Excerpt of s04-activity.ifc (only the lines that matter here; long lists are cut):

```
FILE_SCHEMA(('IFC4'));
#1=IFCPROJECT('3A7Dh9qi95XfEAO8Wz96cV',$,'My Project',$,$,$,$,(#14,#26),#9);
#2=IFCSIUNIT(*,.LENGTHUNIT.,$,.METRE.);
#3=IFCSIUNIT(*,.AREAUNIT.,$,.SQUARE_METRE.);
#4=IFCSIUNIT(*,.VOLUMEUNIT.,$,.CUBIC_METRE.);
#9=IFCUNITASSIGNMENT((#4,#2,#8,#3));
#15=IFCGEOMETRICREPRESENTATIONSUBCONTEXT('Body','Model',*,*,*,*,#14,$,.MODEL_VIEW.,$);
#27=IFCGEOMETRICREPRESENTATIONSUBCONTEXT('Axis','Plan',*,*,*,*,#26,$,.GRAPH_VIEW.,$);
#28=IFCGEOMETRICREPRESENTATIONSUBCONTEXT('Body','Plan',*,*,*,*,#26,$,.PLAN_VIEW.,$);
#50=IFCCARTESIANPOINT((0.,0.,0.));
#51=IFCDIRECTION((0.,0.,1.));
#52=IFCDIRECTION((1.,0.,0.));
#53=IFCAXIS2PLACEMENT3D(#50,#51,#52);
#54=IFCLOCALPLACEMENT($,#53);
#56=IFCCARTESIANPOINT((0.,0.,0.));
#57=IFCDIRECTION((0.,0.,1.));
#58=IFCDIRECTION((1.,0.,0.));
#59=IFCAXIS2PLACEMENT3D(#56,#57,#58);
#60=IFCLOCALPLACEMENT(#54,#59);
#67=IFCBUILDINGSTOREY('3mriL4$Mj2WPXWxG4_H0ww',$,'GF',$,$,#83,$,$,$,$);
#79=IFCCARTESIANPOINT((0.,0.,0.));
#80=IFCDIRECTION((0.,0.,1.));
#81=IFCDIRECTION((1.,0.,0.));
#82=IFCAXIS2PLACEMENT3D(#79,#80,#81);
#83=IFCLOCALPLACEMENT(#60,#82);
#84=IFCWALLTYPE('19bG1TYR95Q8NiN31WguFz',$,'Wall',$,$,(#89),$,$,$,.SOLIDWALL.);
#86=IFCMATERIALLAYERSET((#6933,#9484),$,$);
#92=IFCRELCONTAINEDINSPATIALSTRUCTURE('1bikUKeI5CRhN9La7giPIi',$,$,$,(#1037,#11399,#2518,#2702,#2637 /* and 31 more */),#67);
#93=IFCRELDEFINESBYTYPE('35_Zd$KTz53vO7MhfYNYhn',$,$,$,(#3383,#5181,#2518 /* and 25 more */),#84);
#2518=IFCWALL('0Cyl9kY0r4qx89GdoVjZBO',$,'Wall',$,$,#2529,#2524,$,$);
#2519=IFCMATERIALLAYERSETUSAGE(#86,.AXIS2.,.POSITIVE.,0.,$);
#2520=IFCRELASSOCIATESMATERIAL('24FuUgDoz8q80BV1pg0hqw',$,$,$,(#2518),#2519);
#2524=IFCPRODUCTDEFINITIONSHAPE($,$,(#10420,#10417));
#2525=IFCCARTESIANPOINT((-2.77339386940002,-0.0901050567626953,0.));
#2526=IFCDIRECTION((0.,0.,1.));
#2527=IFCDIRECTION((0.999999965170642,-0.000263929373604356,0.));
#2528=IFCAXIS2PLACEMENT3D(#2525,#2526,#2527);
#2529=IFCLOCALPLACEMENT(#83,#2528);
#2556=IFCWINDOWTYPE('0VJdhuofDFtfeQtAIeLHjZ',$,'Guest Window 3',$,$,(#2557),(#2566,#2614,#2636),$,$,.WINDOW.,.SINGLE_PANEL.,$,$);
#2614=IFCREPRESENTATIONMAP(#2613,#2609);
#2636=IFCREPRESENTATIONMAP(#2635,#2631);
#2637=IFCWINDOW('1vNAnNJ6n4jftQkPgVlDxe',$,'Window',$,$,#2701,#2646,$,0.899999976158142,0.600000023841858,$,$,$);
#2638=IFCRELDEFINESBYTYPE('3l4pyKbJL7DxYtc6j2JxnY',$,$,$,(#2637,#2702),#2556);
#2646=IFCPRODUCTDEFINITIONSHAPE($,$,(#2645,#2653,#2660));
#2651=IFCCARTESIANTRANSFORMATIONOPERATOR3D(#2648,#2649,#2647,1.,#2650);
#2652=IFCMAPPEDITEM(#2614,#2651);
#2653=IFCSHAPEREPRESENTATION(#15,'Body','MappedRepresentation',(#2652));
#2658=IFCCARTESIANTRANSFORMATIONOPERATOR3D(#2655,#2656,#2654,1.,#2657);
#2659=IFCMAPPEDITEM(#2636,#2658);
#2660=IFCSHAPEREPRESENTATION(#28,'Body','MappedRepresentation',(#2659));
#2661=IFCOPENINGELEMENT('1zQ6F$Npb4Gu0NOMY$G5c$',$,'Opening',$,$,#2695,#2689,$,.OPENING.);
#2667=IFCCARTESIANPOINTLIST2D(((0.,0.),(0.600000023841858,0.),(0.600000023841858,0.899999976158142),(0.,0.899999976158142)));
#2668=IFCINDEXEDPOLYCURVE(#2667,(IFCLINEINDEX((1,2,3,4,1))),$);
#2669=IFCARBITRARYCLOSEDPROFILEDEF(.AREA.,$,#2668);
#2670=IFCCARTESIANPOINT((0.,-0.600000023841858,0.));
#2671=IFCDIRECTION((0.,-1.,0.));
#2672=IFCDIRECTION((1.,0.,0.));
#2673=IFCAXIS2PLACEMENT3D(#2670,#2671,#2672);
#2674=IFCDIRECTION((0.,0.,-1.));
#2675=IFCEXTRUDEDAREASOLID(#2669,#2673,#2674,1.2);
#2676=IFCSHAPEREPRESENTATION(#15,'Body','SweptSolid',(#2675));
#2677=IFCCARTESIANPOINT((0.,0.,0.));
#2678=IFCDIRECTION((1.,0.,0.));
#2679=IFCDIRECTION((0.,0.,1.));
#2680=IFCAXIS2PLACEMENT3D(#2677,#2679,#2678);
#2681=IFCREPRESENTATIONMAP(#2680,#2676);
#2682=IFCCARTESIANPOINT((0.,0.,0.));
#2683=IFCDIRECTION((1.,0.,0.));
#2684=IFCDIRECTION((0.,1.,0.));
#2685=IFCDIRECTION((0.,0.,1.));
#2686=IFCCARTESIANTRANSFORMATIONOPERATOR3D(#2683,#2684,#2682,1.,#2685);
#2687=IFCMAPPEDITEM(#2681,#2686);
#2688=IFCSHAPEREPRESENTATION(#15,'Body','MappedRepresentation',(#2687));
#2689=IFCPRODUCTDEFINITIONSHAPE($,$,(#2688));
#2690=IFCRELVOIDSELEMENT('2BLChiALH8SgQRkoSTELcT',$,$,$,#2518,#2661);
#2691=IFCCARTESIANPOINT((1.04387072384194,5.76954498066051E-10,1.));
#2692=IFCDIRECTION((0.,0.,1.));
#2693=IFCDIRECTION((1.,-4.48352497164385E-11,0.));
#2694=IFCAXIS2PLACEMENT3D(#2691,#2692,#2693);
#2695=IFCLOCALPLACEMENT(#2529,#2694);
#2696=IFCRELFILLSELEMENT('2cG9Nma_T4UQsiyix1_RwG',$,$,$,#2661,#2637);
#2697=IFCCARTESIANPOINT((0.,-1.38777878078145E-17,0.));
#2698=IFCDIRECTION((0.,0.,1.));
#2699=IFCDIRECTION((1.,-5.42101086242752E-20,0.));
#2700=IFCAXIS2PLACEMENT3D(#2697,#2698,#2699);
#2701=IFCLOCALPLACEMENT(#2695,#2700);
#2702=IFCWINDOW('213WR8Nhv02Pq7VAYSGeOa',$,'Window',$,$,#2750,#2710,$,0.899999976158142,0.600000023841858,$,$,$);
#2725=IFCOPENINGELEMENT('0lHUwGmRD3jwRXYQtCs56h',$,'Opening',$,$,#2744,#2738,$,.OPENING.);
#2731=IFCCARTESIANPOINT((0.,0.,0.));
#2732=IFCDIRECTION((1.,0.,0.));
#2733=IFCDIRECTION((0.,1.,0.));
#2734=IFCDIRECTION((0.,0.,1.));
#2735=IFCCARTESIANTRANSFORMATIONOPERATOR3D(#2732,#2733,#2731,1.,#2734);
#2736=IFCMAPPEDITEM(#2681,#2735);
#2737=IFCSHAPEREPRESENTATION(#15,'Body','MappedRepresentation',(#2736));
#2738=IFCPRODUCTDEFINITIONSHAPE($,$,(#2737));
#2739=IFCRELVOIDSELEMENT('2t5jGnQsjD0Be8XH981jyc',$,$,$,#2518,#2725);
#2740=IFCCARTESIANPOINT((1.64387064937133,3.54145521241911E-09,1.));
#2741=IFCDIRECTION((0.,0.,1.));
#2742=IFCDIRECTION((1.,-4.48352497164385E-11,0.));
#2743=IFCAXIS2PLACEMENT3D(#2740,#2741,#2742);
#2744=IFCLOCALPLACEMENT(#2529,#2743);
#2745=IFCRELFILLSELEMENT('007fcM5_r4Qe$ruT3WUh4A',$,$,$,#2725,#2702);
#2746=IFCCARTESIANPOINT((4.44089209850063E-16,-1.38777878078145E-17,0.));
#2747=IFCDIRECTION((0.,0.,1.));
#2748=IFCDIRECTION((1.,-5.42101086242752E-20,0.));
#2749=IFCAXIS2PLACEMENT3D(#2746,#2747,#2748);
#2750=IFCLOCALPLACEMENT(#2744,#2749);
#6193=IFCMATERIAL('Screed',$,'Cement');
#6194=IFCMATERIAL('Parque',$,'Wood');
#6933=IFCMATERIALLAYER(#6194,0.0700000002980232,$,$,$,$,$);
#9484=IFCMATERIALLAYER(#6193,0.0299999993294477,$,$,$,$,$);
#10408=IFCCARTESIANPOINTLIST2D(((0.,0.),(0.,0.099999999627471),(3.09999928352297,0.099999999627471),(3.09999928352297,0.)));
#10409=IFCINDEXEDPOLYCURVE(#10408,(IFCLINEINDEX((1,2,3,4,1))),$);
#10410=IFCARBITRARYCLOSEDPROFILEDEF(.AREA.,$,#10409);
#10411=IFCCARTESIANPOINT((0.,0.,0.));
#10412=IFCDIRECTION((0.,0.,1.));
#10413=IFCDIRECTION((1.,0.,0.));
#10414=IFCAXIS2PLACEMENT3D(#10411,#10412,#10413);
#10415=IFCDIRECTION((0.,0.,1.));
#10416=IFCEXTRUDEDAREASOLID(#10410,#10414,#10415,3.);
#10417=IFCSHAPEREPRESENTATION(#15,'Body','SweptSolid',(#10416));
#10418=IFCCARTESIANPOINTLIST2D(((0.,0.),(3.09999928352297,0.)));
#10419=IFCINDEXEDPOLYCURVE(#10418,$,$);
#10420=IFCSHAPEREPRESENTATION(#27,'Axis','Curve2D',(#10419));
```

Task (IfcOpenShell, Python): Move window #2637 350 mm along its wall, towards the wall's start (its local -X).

```python
import ifcopenshell
import ifcopenshell.api.geometry
import ifcopenshell.util.placement
import ifcopenshell.util.unit

model = ifcopenshell.open("s04-activity.ifc")
unit_scale = ifcopenshell.util.unit.calculate_unit_scale(model)

window = model.by_id(2637)
opening = window.FillsVoids[0].RelatingOpeningElement
wall = opening.VoidsElements[0].RelatingBuildingElement

wall_matrix = ifcopenshell.util.placement.get_local_placement(wall.ObjectPlacement)
shift = wall_matrix[:3, 0] * -0.35 / unit_scale
before = ifcopenshell.util.placement.get_local_placement(window.ObjectPlacement)[:3, 3].copy()

# The window is placed relative to its opening, so it follows when the opening moves.
matrix = ifcopenshell.util.placement.get_local_placement(opening.ObjectPlacement)
matrix[:3, 3] += shift
ifcopenshell.api.geometry.edit_object_placement(
    model, product=opening, matrix=matrix, is_si=False, should_transform_children=True
)

after = ifcopenshell.util.placement.get_local_placement(window.ObjectPlacement)[:3, 3]
print("window moved by", (after - before).round(3) + 0.0)

model.write("s04-activity_v2.ifc")
```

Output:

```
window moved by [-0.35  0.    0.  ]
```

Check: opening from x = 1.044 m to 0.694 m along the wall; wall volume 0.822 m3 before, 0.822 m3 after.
